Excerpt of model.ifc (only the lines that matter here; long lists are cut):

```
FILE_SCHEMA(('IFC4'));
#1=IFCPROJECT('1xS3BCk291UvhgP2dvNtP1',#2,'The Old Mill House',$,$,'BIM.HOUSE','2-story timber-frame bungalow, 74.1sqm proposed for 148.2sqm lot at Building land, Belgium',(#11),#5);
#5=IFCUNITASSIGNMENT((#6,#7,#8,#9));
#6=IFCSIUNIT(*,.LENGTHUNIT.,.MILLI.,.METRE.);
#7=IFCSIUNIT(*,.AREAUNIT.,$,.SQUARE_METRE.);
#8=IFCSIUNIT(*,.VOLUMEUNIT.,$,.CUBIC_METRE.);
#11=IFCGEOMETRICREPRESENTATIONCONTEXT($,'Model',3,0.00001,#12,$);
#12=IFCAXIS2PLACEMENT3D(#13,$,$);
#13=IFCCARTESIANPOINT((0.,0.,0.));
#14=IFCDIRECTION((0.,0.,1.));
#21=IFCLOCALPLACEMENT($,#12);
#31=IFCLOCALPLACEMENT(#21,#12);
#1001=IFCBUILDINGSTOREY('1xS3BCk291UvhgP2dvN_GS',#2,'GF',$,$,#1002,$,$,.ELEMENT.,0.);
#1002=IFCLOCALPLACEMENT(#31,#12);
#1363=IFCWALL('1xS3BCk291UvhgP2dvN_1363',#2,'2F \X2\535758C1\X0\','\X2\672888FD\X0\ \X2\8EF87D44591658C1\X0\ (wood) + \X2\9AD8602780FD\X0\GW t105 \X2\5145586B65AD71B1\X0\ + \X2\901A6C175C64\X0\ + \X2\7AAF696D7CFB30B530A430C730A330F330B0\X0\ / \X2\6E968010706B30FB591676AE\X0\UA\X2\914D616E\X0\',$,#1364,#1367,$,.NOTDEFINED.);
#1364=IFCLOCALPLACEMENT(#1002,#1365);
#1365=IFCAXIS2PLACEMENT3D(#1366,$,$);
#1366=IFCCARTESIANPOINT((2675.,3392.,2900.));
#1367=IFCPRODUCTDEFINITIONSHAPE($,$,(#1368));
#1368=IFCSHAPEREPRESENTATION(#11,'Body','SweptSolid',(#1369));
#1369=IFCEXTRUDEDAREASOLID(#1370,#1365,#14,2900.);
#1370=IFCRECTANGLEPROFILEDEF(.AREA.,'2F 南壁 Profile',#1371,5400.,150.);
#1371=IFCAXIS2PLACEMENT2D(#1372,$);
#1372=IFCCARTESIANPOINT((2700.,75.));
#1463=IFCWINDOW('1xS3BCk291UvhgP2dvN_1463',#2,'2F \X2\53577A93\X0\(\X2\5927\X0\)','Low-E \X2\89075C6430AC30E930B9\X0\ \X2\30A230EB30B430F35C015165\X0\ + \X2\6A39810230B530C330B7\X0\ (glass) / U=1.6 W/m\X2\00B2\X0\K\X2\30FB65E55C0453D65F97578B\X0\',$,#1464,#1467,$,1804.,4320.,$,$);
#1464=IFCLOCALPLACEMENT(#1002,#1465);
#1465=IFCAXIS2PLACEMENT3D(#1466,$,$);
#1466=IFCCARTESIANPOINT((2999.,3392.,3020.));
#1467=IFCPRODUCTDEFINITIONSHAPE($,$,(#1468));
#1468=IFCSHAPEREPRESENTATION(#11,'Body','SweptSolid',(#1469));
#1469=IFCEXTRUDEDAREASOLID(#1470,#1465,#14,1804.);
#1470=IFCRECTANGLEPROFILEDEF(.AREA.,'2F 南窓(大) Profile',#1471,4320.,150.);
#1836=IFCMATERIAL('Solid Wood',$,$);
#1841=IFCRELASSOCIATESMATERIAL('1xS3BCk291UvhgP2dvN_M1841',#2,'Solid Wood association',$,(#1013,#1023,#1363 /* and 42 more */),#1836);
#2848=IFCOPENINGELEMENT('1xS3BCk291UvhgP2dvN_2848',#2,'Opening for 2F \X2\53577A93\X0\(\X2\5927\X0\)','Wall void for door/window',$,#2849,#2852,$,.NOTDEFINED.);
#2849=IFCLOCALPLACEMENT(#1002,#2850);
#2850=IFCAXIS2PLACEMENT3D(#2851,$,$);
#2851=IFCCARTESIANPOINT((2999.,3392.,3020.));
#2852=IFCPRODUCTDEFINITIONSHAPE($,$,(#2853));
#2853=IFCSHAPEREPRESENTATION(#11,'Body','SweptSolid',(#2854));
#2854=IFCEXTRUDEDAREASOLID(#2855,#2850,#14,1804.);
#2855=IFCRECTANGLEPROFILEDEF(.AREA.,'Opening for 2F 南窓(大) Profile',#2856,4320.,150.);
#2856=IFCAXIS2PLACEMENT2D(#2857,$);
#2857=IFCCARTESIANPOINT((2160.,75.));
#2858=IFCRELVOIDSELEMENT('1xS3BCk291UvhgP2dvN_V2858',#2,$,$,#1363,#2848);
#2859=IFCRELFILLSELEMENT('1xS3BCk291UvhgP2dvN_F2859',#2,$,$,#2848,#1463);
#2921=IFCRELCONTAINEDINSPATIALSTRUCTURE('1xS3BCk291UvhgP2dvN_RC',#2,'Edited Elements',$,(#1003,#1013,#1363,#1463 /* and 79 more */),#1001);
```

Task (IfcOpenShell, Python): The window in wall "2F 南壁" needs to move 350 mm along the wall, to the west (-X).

```python
import ifcopenshell
import ifcopenshell.api.geometry
import ifcopenshell.util.placement
import ifcopenshell.util.unit

model = ifcopenshell.open("model.ifc")
unit_scale = ifcopenshell.util.unit.calculate_unit_scale(model)

window = model.by_id(1463)
opening = window.FillsVoids[0].RelatingOpeningElement
wall = opening.VoidsElements[0].RelatingBuildingElement

wall_matrix = ifcopenshell.util.placement.get_local_placement(wall.ObjectPlacement)
shift = wall_matrix[:3, 0] * -0.35 / unit_scale
before = ifcopenshell.util.placement.get_local_placement(window.ObjectPlacement)[:3, 3].copy()

# The window is not placed relative to its opening, so move both.
for product in (opening, window):
    matrix = ifcopenshell.util.placement.get_local_placement(product.ObjectPlacement)
    matrix[:3, 3] += shift
    ifcopenshell.api.geometry.edit_object_placement(model, product=product, matrix=matrix, is_si=False)

after = ifcopenshell.util.placement.get_local_placement(window.ObjectPlacement)[:3, 3]
print("window moved by", (after - before).round(3) + 0.0)

model.write("model_rev.ifc")
```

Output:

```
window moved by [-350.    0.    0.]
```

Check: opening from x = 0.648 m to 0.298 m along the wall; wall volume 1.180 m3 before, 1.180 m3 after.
